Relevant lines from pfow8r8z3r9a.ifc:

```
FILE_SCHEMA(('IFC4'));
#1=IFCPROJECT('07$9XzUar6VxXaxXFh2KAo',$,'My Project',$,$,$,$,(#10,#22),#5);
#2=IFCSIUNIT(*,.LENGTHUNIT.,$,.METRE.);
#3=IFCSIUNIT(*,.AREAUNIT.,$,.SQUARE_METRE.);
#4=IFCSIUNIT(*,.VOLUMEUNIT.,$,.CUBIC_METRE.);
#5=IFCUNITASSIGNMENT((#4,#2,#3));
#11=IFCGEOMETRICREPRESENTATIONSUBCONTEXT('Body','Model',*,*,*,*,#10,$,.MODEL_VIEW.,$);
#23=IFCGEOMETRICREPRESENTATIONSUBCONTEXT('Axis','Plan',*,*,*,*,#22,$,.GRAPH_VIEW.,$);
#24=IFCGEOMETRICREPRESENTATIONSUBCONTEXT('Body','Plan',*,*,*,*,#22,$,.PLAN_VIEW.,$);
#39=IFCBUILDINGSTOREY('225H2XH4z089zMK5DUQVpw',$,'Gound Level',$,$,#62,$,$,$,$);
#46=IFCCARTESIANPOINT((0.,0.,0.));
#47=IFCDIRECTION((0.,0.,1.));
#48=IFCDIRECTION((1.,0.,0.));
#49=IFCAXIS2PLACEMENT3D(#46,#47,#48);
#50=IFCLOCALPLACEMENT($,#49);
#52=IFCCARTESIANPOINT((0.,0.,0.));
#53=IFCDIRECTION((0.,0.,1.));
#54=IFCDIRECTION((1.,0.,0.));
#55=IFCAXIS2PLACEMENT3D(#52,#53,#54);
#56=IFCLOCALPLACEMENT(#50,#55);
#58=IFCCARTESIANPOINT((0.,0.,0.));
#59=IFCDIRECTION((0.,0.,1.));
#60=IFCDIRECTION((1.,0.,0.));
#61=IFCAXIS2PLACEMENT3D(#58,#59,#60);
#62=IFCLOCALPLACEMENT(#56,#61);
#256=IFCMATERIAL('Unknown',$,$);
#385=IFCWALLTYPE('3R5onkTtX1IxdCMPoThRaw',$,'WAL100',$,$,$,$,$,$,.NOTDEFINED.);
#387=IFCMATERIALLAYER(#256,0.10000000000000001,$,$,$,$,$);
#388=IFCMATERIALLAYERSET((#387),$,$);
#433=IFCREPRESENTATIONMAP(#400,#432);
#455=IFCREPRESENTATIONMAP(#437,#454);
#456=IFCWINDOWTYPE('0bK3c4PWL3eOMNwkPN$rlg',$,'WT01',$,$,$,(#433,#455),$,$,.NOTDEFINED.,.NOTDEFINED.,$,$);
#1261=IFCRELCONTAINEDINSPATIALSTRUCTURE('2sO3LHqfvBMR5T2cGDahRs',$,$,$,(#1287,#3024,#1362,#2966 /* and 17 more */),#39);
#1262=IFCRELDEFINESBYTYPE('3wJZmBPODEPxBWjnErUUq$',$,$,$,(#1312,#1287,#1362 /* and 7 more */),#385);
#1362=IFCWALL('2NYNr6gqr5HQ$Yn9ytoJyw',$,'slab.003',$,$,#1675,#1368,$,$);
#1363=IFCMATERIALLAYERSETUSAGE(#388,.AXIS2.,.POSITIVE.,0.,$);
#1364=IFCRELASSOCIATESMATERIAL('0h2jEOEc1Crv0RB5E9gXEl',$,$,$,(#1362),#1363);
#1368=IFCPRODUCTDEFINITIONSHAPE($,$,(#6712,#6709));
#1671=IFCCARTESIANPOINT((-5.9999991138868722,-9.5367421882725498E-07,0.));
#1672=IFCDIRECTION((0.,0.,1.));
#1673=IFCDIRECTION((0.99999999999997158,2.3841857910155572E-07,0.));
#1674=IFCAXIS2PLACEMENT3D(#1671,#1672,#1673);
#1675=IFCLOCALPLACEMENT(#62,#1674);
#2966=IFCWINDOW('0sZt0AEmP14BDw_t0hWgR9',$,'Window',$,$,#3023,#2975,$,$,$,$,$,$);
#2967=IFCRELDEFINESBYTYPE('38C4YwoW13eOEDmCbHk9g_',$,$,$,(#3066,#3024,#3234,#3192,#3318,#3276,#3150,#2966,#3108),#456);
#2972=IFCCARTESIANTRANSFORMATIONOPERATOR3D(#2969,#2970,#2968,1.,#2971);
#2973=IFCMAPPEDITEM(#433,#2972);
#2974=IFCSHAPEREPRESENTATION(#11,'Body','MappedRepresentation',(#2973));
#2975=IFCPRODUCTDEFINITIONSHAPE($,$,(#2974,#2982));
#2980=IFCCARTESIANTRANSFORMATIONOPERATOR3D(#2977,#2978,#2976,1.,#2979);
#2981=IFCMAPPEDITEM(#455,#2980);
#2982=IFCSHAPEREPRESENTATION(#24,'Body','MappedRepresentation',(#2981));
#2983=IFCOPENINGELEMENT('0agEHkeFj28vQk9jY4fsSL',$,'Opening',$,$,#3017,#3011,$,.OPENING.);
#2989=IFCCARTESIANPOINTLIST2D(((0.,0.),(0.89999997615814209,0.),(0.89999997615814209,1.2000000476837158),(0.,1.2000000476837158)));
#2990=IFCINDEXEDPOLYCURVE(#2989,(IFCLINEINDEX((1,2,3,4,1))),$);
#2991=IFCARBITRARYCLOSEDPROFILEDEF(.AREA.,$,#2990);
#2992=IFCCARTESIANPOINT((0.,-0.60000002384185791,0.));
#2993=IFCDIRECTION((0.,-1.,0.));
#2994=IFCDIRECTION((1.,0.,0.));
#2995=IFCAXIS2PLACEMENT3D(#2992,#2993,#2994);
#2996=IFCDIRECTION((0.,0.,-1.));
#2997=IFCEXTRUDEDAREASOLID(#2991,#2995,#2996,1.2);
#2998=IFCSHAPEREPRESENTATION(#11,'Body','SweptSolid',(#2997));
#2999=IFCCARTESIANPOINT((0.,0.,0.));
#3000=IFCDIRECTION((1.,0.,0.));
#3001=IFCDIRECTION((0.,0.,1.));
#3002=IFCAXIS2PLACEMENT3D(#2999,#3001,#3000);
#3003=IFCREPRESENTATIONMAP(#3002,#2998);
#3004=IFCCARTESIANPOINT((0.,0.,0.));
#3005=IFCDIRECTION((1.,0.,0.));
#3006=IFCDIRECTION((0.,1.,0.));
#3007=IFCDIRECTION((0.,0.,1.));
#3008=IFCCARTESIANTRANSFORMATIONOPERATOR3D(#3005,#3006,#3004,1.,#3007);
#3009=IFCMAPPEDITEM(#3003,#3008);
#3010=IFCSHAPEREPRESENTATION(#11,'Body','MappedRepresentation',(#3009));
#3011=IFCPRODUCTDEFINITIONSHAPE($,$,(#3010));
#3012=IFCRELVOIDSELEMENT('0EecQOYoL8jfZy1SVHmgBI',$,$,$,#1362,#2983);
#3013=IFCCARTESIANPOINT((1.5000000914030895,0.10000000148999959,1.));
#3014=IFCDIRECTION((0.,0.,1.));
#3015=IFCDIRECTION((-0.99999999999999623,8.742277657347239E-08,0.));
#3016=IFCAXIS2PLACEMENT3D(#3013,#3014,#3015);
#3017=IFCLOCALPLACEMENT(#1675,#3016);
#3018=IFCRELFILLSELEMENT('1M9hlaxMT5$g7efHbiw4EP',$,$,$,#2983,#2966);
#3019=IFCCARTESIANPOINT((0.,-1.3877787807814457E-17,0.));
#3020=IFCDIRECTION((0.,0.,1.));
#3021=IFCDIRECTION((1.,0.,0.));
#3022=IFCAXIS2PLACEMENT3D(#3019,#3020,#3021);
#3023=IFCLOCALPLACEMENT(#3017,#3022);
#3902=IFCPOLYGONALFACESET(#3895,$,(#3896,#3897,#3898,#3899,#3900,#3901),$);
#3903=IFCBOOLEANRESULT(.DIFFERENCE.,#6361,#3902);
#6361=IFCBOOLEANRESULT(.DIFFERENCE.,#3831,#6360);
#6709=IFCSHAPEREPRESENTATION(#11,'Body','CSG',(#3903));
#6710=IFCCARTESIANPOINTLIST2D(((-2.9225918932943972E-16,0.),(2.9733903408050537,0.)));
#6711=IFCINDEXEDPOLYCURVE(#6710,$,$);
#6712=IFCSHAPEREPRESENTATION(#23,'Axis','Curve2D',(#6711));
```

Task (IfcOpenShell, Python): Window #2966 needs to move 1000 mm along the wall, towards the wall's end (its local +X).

```python
import ifcopenshell
import ifcopenshell.api.geometry
import ifcopenshell.util.placement

model = ifcopenshell.open("pfow8r8z3r9a.ifc")

window = model.by_guid("0sZt0AEmP14BDw_t0hWgR9")
opening = window.FillsVoids[0].RelatingOpeningElement
wall = opening.VoidsElements[0].RelatingBuildingElement

wall_matrix = ifcopenshell.util.placement.get_local_placement(wall.ObjectPlacement)
shift = wall_matrix[:3, 0] * 1.0
before = ifcopenshell.util.placement.get_local_placement(window.ObjectPlacement)[:3, 3].copy()

# The window is placed relative to its opening, so it follows when the opening moves.
matrix = ifcopenshell.util.placement.get_local_placement(opening.ObjectPlacement)
matrix[:3, 3] += shift
ifcopenshell.api.geometry.edit_object_placement(
    model, product=opening, matrix=matrix, is_si=False, should_transform_children=True
)

after = ifcopenshell.util.placement.get_local_placement(window.ObjectPlacement)[:3, 3]
print("window moved by", (after - before).round(3) + 0.0)

model.write("pfow8r8z3r9a_updated.ifc")
```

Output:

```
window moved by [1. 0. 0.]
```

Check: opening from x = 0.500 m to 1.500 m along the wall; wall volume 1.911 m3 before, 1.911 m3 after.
